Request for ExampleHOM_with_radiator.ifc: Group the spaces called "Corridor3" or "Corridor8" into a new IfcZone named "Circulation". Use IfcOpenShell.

First a look at what the model holds.

```python
import ifcopenshell

model = ifcopenshell.open("ExampleHOM_with_radiator.ifc")
print(model.schema)
seen = {}
for space in model.by_type("IfcSpace"):
    seen[space.Name] = seen.get(space.Name, 0) + 1
for name, count in sorted(seen.items(), key=str):
    print(count, "x", name)
print("zones:", [z.Name for z in model.by_type("IfcZone")][:20])
```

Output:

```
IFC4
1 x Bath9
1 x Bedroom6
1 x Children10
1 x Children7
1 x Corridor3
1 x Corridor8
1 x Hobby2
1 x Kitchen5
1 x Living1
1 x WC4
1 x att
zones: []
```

```python
import ifcopenshell
import ifcopenshell.api.group
import ifcopenshell.api.root

model = ifcopenshell.open("ExampleHOM_with_radiator.ifc")

names = {"Corridor3", "Corridor8"}
spaces = [s for s in model.by_type("IfcSpace") if s.Name in names]

zone = ifcopenshell.api.root.create_entity(model, ifc_class="IfcZone", name="Circulation")
ifcopenshell.api.group.assign_group(model, products=spaces, group=zone)
print(len(spaces), "spaces in", zone.Name)

model.write("ExampleHOM_with_radiator_v2.ifc")
```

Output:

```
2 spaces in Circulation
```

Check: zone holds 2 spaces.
